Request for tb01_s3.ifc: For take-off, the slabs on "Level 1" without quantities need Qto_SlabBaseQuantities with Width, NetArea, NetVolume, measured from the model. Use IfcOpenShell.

First a look at what the model holds.

```python
import ifcopenshell
import ifcopenshell.util.element
import ifcopenshell.util.unit

model = ifcopenshell.open("tb01_s3.ifc")
print(model.schema)
for unit_type in ("LENGTHUNIT", "AREAUNIT", "VOLUMEUNIT"):
    print(unit_type, ifcopenshell.util.unit.calculate_unit_scale(model, unit_type))
storey = next(s for s in model.by_type("IfcBuildingStorey") if s.Name == "Level 1")
slabs = [e for e in ifcopenshell.util.element.get_decomposition(storey) if e.is_a("IfcSlab")]
for e in sorted(slabs, key=lambda e: e.id()):
    print(e.id(), e.is_a(), e.Name, list(ifcopenshell.util.element.get_psets(e, qtos_only=True)), sep=" | ")
```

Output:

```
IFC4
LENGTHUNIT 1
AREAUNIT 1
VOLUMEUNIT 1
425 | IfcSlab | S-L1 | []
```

```python
import ifcopenshell
import ifcopenshell.api.pset
import ifcopenshell.geom
import ifcopenshell.util.element
import ifcopenshell.util.shape
import ifcopenshell.util.unit

model = ifcopenshell.open("tb01_s3.ifc")
unit_scale = ifcopenshell.util.unit.calculate_unit_scale(model)
area_scale = ifcopenshell.util.unit.calculate_unit_scale(model, "AREAUNIT")
volume_scale = ifcopenshell.util.unit.calculate_unit_scale(model, "VOLUMEUNIT")
settings = ifcopenshell.geom.settings()

storey = next(s for s in model.by_type("IfcBuildingStorey") if s.Name == "Level 1")
slabs = [e for e in ifcopenshell.util.element.get_decomposition(storey) if e.is_a("IfcSlab")]

for e in sorted(slabs, key=lambda e: e.id()):
    if ifcopenshell.util.element.get_psets(e, qtos_only=True, should_inherit=False):
        continue
    # Geometry comes back in metres, in the element's own axes.
    shape = ifcopenshell.geom.create_shape(settings, e)
    values = {
        "Width": ifcopenshell.util.shape.get_z(shape.geometry) / unit_scale,
        "NetArea": ifcopenshell.util.shape.get_footprint_area(shape.geometry) / area_scale,
        "NetVolume": ifcopenshell.util.shape.get_volume(shape.geometry) / volume_scale,
    }
    qto = ifcopenshell.api.pset.add_qto(model, product=e, name="Qto_SlabBaseQuantities")
    ifcopenshell.api.pset.edit_qto(model, qto=qto, properties=values)
    print(e.id(), {k: round(v, 3) for k, v in values.items()})

model.write("tb01_s3_v2.ifc")
```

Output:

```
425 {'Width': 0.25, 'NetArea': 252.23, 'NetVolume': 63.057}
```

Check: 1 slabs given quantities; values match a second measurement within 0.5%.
